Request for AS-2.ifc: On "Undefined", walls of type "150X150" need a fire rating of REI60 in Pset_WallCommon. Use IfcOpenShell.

First a look at what the model holds.

```python
import ifcopenshell
import ifcopenshell.util.element

model = ifcopenshell.open("AS-2.ifc")
print(model.schema)
storey = next(s for s in model.by_type("IfcBuildingStorey") if s.Name == "Undefined")
walls = [e for e in ifcopenshell.util.element.get_decomposition(storey) if e.is_a("IfcWall")]
seen = {}
for e in walls:
    element_type = ifcopenshell.util.element.get_type(e)
    key = (element_type.Name if element_type != e and element_type else None, ifcopenshell.util.element.get_pset(e, "Pset_WallCommon", "FireRating"))
    seen[key] = seen.get(key, 0) + 1
for (name, value), count in sorted(seen.items(), key=str):
    print(count, "x", name, "|", value)
```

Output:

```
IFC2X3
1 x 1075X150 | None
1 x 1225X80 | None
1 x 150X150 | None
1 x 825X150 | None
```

```python
import ifcopenshell
import ifcopenshell.api.pset
import ifcopenshell.util.element

model = ifcopenshell.open("AS-2.ifc")

storey = next(s for s in model.by_type("IfcBuildingStorey") if s.Name == "Undefined")
walls = [e for e in ifcopenshell.util.element.get_decomposition(storey) if e.is_a("IfcWall")]

count = 0
for e in walls:
    element_type = ifcopenshell.util.element.get_type(e)
    if element_type in (None, e) or element_type.Name != "150X150":
        continue
    # add_pset returns the element's existing set when there is one.
    pset = ifcopenshell.api.pset.add_pset(model, product=e, name="Pset_WallCommon")
    ifcopenshell.api.pset.edit_pset(model, pset=pset, properties={"FireRating": "REI60"})
    count += 1

print(count, "walls updated")

model.write("AS-2-out.ifc")
```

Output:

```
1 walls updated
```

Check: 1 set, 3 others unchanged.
